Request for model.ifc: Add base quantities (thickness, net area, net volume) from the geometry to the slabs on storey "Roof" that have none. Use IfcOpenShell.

First a look at what the model holds.

```python
import ifcopenshell
import ifcopenshell.util.element
import ifcopenshell.util.unit

model = ifcopenshell.open("model.ifc")
print(model.schema)
for unit_type in ("LENGTHUNIT", "AREAUNIT", "VOLUMEUNIT"):
    print(unit_type, ifcopenshell.util.unit.calculate_unit_scale(model, unit_type))
storey = next(s for s in model.by_type("IfcBuildingStorey") if s.Name == "Roof")
slabs = [e for e in ifcopenshell.util.element.get_decomposition(storey) if e.is_a("IfcSlab")]
for e in sorted(slabs, key=lambda e: e.id()):
    print(e.id(), e.is_a(), e.Name, list(ifcopenshell.util.element.get_psets(e, qtos_only=True)), sep=" | ")
```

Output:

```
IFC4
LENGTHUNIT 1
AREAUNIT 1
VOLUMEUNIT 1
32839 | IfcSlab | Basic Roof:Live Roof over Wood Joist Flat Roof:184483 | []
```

```python
import ifcopenshell
import ifcopenshell.api.pset
import ifcopenshell.geom
import ifcopenshell.util.element
import ifcopenshell.util.shape
import ifcopenshell.util.unit

model = ifcopenshell.open("model.ifc")
unit_scale = ifcopenshell.util.unit.calculate_unit_scale(model)
area_scale = ifcopenshell.util.unit.calculate_unit_scale(model, "AREAUNIT")
volume_scale = ifcopenshell.util.unit.calculate_unit_scale(model, "VOLUMEUNIT")
settings = ifcopenshell.geom.settings()

storey = next(s for s in model.by_type("IfcBuildingStorey") if s.Name == "Roof")
slabs = [e for e in ifcopenshell.util.element.get_decomposition(storey) if e.is_a("IfcSlab")]

for e in sorted(slabs, key=lambda e: e.id()):
    if ifcopenshell.util.element.get_psets(e, qtos_only=True, should_inherit=False):
        continue
    # Geometry comes back in metres, in the element's own axes.
    shape = ifcopenshell.geom.create_shape(settings, e)
    values = {
        "Width": ifcopenshell.util.shape.get_z(shape.geometry) / unit_scale,
        "NetArea": ifcopenshell.util.shape.get_footprint_area(shape.geometry) / area_scale,
        "NetVolume": ifcopenshell.util.shape.get_volume(shape.geometry) / volume_scale,
    }
    qto = ifcopenshell.api.pset.add_qto(model, product=e, name="Qto_SlabBaseQuantities")
    ifcopenshell.api.pset.edit_qto(model, qto=qto, properties=values)
    print(e.id(), {k: round(v, 3) for k, v in values.items()})

model.write("model_edited.ifc")
```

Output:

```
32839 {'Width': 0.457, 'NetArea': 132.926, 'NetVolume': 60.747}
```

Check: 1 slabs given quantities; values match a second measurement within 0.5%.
